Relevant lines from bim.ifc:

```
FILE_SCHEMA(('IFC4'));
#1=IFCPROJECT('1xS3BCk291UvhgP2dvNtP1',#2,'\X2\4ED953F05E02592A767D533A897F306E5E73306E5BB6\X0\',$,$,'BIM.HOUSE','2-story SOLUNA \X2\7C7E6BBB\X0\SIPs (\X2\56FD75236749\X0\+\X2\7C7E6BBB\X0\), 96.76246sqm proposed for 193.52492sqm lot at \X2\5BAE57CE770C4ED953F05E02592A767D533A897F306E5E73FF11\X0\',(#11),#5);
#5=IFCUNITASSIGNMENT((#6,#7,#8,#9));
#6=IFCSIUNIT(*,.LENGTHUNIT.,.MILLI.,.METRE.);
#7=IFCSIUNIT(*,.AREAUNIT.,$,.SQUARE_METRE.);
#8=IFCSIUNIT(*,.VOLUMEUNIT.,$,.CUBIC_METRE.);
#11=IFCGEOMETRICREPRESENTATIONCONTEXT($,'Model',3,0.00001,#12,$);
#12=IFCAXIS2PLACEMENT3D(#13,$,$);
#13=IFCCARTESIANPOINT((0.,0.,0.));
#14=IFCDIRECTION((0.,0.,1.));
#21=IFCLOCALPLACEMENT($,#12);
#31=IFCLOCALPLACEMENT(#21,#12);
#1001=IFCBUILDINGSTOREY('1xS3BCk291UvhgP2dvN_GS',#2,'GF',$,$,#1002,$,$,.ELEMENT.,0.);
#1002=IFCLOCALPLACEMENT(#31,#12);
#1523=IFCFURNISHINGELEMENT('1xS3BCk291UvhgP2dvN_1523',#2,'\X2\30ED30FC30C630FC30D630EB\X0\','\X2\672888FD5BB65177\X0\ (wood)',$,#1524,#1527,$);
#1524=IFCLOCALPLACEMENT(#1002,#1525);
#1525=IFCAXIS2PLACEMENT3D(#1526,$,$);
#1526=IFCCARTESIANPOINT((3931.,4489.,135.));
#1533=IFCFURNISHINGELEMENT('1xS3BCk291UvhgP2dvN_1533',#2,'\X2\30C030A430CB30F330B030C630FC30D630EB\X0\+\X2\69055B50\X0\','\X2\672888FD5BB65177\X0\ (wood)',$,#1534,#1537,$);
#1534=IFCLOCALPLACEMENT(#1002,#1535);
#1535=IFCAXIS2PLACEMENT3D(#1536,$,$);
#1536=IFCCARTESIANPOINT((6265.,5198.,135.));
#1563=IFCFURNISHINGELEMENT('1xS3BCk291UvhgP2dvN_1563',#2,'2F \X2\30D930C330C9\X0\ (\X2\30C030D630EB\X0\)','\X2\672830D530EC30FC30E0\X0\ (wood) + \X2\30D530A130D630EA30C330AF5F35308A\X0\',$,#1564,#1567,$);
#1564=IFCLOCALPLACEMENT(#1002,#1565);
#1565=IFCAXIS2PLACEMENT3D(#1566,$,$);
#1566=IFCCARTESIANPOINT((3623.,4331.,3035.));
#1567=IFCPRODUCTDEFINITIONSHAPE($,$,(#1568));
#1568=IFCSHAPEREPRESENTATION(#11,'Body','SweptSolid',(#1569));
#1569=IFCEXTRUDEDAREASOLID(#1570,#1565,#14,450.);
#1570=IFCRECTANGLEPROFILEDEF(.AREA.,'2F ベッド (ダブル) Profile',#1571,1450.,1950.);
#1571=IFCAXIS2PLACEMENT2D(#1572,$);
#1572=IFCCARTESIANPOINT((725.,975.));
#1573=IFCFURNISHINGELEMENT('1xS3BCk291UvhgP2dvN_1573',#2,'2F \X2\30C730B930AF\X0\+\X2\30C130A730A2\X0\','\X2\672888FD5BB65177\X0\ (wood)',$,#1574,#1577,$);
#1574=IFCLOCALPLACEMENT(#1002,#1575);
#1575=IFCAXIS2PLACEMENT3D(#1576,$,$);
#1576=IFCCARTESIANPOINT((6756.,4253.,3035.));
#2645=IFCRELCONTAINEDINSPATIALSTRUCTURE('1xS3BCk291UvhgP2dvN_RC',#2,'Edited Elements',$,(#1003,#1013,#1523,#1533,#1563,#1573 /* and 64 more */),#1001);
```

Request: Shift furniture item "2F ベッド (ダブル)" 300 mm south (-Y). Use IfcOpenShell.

```python
import ifcopenshell
import ifcopenshell.api.geometry
import ifcopenshell.util.placement
import ifcopenshell.util.unit

model = ifcopenshell.open("bim.ifc")
unit_scale = ifcopenshell.util.unit.calculate_unit_scale(model)

item = model.by_id(1563)
matrix = ifcopenshell.util.placement.get_local_placement(item.ObjectPlacement)
matrix[1, 3] -= 0.3 / unit_scale
ifcopenshell.api.geometry.edit_object_placement(model, product=item, matrix=matrix, is_si=False)

print(ifcopenshell.util.placement.get_local_placement(item.ObjectPlacement).round(3) + 0.0)

model.write("bim_rev.ifc")
```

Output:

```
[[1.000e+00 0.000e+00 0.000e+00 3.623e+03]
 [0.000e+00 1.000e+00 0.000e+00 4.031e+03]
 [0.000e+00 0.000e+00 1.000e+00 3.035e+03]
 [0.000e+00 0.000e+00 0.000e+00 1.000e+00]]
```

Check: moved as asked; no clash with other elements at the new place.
